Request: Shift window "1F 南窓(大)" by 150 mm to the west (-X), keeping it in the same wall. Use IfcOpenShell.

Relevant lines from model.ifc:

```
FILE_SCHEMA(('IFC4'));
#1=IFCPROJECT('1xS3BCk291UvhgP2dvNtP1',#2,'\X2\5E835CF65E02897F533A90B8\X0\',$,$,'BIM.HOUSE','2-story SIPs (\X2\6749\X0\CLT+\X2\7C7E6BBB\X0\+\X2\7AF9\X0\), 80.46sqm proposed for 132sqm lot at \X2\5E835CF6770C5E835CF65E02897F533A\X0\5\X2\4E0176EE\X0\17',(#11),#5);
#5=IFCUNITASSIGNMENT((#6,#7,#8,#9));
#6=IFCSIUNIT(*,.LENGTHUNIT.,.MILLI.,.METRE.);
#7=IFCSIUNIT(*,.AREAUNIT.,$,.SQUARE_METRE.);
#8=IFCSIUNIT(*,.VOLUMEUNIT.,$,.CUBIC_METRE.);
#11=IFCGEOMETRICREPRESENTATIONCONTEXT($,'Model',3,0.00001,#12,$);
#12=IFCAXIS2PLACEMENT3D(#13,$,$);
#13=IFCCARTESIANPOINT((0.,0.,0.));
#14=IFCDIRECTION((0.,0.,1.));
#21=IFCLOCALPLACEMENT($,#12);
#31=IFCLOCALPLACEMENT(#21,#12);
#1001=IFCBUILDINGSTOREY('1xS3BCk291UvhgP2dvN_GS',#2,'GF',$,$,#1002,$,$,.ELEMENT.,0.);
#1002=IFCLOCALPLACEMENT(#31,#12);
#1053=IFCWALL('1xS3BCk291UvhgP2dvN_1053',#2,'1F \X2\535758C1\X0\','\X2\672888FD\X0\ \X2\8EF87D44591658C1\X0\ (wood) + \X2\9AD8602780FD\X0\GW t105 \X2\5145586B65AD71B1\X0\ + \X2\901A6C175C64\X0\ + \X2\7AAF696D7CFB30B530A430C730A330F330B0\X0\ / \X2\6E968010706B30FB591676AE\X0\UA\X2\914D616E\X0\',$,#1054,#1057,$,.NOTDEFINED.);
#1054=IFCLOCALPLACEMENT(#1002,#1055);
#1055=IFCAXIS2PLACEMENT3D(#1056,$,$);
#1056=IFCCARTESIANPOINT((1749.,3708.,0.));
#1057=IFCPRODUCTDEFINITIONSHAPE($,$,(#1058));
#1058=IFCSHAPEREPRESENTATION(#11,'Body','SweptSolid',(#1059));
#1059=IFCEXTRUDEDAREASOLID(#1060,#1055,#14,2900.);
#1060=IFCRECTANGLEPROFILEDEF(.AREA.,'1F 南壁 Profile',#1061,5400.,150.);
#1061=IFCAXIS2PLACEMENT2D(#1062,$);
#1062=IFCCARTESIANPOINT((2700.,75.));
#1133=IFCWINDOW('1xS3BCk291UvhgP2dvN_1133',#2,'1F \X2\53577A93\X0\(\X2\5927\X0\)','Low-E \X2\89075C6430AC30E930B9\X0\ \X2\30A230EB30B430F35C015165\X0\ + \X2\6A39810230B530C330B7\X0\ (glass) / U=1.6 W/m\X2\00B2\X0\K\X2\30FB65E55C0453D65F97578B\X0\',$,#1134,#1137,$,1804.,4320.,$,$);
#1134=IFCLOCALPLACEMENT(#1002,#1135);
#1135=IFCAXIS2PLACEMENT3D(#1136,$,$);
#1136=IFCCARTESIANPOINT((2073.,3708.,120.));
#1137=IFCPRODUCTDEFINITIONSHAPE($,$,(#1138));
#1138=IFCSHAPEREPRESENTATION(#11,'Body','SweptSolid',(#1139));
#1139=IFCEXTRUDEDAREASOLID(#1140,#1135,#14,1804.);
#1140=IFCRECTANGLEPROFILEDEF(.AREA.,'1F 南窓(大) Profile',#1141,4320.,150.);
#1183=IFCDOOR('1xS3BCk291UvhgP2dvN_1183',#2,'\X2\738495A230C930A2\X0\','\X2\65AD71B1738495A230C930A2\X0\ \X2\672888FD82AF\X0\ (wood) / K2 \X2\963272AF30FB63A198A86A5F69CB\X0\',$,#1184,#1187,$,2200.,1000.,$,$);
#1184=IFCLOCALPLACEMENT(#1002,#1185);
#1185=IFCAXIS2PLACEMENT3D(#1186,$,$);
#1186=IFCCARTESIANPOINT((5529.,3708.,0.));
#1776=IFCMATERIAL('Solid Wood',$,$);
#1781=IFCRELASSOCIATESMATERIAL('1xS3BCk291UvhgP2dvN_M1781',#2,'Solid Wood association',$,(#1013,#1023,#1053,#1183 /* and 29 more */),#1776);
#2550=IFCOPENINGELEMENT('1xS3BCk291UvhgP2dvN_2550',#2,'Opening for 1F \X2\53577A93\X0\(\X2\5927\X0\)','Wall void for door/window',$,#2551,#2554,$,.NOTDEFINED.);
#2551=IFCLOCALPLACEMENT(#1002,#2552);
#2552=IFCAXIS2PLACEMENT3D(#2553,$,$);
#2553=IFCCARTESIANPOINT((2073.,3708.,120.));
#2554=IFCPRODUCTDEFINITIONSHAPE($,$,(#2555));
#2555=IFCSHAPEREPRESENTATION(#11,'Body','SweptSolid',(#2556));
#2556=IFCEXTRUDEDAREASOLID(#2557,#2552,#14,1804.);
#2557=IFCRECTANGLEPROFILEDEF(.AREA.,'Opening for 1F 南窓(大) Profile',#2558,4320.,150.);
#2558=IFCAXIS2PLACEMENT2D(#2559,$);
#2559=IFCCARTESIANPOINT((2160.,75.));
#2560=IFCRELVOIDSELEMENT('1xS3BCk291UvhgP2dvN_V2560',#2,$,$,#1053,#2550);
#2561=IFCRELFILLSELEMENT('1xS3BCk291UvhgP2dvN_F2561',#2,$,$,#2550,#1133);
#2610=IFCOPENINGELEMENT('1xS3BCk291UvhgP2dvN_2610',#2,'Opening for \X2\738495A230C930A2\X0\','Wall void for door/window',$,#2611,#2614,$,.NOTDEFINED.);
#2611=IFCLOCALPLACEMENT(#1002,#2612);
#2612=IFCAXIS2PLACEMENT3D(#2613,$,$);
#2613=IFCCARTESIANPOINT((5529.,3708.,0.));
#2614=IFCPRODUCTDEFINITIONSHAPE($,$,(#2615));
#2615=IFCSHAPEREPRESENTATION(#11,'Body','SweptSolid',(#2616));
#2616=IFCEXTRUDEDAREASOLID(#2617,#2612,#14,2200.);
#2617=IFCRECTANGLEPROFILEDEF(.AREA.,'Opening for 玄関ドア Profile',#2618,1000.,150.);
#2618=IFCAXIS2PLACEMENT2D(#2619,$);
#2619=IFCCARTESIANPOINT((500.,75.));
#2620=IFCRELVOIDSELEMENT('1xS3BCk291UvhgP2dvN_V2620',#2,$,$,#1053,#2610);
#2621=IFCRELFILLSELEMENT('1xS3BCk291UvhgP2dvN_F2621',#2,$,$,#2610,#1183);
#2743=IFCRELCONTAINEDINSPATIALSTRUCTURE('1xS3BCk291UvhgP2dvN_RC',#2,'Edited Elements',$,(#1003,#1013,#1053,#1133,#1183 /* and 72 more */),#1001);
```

```python
import ifcopenshell
import ifcopenshell.api.geometry
import ifcopenshell.util.placement

model = ifcopenshell.open("model.ifc")

window = model.by_guid("1xS3BCk291UvhgP2dvN_1133")
opening = window.FillsVoids[0].RelatingOpeningElement
wall = opening.VoidsElements[0].RelatingBuildingElement

wall_matrix = ifcopenshell.util.placement.get_local_placement(wall.ObjectPlacement)
shift = wall_matrix[:3, 0] * -150.0
before = ifcopenshell.util.placement.get_local_placement(window.ObjectPlacement)[:3, 3].copy()

# The window is not placed relative to its opening, so move both.
for product in (opening, window):
    matrix = ifcopenshell.util.placement.get_local_placement(product.ObjectPlacement)
    matrix[:3, 3] += shift
    ifcopenshell.api.geometry.edit_object_placement(model, product=product, matrix=matrix, is_si=False)

after = ifcopenshell.util.placement.get_local_placement(window.ObjectPlacement)[:3, 3]
print("window moved by", (after - before).round(3) + 0.0)

model.write("model_updated.ifc")
```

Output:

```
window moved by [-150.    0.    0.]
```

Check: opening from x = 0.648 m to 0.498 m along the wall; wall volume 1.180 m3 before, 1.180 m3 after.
